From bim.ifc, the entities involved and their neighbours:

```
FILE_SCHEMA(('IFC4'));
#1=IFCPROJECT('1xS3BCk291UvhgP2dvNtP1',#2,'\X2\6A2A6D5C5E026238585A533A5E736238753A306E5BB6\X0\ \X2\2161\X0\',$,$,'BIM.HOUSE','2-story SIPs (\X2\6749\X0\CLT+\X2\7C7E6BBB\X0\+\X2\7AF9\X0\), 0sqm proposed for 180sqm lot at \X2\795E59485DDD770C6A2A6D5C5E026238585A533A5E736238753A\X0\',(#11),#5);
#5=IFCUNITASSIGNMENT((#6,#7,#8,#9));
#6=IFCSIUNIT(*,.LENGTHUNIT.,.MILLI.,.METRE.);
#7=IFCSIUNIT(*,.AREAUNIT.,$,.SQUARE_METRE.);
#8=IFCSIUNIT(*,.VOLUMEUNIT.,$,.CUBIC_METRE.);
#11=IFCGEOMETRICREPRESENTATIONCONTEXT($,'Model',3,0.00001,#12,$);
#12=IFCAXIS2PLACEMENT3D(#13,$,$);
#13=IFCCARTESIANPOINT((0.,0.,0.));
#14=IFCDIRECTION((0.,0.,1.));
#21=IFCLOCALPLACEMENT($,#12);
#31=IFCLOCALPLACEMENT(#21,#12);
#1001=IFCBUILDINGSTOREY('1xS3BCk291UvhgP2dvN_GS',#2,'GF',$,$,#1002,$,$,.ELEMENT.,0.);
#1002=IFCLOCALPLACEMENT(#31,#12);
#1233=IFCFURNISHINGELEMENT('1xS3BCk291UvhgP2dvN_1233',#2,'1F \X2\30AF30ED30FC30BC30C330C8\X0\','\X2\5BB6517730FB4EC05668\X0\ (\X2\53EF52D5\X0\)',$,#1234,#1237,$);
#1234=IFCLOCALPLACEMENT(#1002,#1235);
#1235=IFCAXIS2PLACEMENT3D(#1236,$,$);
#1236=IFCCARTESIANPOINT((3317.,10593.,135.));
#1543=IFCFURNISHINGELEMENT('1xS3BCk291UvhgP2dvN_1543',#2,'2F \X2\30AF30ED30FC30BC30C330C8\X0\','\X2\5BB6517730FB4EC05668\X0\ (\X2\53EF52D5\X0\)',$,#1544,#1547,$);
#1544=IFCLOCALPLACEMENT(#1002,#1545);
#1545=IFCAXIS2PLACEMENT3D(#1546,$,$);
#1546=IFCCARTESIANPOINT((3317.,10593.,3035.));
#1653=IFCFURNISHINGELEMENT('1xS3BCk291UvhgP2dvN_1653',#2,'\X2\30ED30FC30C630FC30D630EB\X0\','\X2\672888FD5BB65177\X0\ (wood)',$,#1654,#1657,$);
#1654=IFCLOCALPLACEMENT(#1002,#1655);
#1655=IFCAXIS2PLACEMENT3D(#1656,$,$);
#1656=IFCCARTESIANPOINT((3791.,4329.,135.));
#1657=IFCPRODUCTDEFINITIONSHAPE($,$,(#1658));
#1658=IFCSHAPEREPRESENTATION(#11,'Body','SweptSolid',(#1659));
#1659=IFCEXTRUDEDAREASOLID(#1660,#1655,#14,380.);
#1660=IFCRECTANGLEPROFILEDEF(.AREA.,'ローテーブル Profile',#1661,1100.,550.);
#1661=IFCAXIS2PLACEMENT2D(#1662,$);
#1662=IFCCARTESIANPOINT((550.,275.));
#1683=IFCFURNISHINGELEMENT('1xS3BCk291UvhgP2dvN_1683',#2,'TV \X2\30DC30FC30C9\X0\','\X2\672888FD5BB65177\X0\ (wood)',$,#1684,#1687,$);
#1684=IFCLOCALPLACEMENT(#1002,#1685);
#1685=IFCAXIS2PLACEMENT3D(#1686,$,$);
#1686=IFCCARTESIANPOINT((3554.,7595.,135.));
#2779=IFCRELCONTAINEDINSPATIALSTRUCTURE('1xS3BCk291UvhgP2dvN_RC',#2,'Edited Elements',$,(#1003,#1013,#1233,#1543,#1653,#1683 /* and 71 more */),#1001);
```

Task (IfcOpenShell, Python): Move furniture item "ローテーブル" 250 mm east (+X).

```python
import ifcopenshell
import ifcopenshell.api.geometry
import ifcopenshell.util.placement

model = ifcopenshell.open("bim.ifc")

item = model.by_guid("1xS3BCk291UvhgP2dvN_1653")
matrix = ifcopenshell.util.placement.get_local_placement(item.ObjectPlacement)
matrix[0, 3] += 250.0
ifcopenshell.api.geometry.edit_object_placement(model, product=item, matrix=matrix, is_si=False)

print(ifcopenshell.util.placement.get_local_placement(item.ObjectPlacement).round(3) + 0.0)

model.write("bim_rev.ifc")
```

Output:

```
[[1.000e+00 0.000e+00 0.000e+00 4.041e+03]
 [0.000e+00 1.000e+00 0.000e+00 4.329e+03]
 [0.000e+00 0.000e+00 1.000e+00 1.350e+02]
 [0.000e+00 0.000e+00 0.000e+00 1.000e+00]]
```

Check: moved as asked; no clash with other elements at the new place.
